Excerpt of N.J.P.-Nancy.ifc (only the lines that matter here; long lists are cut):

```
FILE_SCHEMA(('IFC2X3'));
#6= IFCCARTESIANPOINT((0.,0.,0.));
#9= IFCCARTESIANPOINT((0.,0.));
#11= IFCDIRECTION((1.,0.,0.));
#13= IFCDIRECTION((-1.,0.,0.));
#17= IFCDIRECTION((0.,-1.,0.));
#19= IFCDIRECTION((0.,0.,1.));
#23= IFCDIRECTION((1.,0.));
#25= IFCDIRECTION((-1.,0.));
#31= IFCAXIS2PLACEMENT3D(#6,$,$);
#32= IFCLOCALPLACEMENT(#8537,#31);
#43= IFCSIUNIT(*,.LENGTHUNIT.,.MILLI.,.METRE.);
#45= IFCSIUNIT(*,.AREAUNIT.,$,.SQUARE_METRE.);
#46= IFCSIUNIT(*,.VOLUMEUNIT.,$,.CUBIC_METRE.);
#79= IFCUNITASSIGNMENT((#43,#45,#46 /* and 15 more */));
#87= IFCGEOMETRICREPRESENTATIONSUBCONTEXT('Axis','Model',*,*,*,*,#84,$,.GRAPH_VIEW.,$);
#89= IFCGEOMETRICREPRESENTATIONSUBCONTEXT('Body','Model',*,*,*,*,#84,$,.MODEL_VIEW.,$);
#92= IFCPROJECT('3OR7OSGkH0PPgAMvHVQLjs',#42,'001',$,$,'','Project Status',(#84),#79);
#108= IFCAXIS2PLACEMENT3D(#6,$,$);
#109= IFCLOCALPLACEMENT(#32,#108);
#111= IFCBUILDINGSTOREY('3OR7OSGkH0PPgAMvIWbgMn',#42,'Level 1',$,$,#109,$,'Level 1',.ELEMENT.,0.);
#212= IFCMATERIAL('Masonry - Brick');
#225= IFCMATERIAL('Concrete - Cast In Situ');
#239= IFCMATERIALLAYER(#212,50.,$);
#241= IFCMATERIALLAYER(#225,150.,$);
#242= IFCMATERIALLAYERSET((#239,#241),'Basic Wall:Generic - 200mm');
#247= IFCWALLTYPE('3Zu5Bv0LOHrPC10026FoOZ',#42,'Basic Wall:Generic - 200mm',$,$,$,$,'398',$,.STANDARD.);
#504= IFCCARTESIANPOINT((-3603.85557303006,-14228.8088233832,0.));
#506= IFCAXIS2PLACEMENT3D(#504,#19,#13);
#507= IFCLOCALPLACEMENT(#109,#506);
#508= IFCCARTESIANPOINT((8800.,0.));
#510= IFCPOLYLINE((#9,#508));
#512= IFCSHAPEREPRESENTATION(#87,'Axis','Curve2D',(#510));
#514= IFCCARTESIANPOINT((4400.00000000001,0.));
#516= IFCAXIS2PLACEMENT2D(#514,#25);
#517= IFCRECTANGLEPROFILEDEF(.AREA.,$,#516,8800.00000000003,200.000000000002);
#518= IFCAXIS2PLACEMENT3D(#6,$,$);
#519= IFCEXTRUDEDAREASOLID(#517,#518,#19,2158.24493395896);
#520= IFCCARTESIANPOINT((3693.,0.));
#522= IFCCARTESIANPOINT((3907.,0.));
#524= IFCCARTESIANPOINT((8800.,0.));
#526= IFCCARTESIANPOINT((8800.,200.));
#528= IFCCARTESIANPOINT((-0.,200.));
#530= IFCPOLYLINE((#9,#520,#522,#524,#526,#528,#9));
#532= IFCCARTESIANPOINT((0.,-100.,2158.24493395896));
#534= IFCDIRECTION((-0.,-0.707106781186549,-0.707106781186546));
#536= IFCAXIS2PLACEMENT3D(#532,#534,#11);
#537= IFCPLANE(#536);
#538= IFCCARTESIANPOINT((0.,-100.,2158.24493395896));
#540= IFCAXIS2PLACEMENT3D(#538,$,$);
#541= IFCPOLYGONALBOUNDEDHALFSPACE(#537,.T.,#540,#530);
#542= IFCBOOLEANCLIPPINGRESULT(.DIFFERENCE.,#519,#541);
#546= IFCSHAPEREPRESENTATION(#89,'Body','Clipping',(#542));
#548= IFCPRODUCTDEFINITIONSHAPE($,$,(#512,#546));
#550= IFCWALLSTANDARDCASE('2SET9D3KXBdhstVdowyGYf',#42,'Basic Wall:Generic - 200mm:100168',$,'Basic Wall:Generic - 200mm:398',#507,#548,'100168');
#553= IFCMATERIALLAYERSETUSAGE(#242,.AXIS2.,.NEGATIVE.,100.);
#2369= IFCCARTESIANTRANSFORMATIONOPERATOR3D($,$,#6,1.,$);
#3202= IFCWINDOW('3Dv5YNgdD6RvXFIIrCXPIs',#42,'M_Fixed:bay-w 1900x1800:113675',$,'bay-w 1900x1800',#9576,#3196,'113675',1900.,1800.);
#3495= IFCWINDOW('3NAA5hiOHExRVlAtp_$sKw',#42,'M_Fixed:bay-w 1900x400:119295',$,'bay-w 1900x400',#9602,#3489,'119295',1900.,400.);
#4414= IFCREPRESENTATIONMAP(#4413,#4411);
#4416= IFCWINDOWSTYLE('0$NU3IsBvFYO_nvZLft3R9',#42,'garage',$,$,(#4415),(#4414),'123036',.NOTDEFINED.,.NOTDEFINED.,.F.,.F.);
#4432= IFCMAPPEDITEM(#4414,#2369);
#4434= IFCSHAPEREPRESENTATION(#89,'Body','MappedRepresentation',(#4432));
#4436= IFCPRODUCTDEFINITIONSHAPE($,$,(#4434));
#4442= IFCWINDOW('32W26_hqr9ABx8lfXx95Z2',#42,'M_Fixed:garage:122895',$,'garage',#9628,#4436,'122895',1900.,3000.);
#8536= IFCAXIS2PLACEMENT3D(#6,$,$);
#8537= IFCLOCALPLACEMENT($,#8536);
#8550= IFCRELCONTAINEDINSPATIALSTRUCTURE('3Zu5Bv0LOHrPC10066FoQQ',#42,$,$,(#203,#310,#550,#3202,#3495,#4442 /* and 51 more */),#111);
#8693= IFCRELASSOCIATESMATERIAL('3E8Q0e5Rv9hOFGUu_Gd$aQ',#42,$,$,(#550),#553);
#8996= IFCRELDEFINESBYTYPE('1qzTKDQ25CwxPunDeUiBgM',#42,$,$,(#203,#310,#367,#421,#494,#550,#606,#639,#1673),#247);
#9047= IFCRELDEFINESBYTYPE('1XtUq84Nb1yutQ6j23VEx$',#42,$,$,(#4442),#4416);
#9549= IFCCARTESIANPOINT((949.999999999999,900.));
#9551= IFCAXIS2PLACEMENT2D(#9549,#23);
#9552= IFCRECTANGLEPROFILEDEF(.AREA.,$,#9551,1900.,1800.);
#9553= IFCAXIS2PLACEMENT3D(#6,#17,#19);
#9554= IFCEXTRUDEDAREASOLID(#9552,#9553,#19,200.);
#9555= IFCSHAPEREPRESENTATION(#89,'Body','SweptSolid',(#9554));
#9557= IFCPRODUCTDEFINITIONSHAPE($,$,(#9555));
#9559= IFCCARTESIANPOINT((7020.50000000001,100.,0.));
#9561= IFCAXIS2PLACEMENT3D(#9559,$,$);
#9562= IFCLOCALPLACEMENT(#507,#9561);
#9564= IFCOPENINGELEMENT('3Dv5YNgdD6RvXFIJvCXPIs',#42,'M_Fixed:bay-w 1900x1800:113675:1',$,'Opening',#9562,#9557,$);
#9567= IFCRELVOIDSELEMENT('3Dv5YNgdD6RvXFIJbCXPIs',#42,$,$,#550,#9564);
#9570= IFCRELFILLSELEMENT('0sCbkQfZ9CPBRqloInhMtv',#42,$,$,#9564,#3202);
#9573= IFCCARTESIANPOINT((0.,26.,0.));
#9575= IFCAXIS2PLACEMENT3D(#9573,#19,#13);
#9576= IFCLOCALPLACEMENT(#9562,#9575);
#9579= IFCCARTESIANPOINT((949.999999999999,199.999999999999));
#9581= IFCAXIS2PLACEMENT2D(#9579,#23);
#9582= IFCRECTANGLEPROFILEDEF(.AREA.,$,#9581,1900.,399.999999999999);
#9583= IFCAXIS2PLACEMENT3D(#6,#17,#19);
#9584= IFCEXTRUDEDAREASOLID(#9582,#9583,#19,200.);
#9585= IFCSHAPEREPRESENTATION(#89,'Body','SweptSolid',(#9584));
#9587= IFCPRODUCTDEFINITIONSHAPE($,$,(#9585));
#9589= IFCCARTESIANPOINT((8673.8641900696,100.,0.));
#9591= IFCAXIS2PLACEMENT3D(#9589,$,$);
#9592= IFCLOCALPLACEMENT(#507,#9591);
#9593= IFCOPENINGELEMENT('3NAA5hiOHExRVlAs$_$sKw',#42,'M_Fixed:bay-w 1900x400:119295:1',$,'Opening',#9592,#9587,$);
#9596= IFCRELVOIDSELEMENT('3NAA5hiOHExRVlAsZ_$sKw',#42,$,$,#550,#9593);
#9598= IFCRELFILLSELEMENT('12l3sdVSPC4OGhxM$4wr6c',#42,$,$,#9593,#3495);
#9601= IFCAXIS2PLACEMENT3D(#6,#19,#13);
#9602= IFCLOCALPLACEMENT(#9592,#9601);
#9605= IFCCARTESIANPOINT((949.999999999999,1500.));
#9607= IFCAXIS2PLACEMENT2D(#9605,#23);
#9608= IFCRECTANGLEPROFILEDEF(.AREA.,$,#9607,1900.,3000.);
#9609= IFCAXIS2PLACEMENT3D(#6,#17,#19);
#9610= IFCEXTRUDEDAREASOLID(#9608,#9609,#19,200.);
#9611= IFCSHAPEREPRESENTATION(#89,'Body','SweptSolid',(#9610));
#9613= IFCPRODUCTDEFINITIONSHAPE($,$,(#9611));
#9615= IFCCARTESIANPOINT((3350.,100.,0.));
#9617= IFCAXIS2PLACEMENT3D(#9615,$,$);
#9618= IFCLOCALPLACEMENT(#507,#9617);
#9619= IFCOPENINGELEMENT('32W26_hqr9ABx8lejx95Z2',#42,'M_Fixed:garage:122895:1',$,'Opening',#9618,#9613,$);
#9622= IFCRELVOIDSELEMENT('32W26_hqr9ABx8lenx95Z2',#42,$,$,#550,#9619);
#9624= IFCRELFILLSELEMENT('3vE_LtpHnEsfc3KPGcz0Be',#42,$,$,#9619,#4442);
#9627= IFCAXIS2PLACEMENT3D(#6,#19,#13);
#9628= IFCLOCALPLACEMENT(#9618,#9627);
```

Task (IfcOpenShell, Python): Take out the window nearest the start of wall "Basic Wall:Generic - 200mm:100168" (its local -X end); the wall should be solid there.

```python
import ifcopenshell
import ifcopenshell.api.feature
import ifcopenshell.api.root
import ifcopenshell.geom
import ifcopenshell.util.shape

model = ifcopenshell.open("N.J.P.-Nancy.ifc")
settings = ifcopenshell.geom.settings()


def volume(element):
    """Net volume in cubic metres, openings subtracted."""
    shape = ifcopenshell.geom.create_shape(settings, element)
    return ifcopenshell.util.shape.get_volume(shape.geometry)


window = model.by_guid("32W26_hqr9ABx8lfXx95Z2")
opening = window.FillsVoids[0].RelatingOpeningElement
wall = opening.VoidsElements[0].RelatingBuildingElement
before = volume(wall)

ifcopenshell.api.root.remove_product(model, product=window)
ifcopenshell.api.feature.remove_feature(model, feature=opening)

after = volume(wall)

print(f"wall volume {before:.3f} -> {after:.3f} m3")

model.write("N.J.P.-Nancy_v2.ifc")
```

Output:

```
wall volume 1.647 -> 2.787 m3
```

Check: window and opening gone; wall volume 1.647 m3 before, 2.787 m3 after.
